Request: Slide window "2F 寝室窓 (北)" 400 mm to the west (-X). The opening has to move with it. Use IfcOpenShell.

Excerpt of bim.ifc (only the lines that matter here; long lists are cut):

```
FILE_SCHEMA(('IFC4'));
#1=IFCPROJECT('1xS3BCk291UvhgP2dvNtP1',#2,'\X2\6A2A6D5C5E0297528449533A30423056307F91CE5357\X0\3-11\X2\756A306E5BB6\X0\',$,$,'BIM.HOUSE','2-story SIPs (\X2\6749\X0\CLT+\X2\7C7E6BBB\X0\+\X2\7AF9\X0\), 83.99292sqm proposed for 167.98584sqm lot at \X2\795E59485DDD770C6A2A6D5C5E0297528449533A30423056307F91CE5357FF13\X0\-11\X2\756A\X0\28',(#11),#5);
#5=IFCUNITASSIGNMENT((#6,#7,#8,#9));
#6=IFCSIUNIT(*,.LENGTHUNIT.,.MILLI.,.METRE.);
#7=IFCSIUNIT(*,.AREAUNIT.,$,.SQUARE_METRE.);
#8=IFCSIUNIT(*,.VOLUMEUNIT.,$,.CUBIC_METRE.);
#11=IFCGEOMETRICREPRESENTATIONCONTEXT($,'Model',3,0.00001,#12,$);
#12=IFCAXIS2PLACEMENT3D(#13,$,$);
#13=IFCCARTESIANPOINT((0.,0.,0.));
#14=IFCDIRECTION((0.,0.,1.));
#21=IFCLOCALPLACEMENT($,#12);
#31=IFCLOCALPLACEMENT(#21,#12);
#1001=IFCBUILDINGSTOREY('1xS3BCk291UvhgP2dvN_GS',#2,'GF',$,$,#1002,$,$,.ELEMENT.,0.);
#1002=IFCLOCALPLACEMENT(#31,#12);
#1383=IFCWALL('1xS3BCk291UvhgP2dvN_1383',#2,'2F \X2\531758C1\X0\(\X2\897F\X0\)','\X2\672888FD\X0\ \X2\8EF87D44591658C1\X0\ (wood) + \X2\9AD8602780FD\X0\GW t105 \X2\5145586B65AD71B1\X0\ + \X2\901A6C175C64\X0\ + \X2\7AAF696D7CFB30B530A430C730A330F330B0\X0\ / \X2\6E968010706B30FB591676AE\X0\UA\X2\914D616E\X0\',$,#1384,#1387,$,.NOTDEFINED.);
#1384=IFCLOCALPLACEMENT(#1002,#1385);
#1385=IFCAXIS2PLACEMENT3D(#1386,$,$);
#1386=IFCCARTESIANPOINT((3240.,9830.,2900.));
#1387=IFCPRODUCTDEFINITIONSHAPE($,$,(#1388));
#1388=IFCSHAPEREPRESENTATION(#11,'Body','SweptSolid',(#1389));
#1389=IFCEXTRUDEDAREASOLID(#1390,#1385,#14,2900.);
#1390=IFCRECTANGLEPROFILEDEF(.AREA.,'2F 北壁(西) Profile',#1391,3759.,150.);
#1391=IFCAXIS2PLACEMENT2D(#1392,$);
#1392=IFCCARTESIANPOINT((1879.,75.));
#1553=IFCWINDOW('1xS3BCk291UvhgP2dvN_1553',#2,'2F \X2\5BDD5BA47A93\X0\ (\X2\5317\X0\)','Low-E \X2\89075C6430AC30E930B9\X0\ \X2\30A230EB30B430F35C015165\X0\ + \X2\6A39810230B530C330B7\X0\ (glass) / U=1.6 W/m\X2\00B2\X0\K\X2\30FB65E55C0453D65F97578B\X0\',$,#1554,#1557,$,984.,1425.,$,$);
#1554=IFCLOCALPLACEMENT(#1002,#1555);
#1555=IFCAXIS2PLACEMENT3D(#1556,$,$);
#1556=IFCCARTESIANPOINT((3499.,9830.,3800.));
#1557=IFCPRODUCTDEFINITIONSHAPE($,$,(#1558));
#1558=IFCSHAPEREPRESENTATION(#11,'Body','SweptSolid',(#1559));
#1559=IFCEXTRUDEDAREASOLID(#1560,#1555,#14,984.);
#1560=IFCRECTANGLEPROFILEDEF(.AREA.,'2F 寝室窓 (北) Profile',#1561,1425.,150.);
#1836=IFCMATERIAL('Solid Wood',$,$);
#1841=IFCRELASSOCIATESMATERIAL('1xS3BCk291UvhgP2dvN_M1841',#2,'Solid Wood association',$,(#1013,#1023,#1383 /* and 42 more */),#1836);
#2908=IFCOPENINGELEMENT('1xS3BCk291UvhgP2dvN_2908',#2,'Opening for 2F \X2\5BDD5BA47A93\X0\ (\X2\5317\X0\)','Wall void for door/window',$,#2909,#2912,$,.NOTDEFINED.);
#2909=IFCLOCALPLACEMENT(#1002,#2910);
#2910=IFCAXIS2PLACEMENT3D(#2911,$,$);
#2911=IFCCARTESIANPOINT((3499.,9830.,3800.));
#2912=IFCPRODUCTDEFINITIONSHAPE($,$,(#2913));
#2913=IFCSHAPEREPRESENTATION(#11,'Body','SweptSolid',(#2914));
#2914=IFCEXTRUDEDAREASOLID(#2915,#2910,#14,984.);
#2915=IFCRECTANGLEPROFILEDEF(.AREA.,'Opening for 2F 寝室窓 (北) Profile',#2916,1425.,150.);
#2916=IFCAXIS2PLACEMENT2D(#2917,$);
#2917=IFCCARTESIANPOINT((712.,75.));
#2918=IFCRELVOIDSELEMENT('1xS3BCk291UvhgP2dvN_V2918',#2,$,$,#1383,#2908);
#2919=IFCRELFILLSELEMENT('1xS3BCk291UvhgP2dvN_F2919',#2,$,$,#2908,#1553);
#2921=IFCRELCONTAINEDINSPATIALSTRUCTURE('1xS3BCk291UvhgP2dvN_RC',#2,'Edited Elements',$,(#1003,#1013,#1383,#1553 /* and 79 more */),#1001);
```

```python
import ifcopenshell
import ifcopenshell.api.geometry
import ifcopenshell.util.placement

model = ifcopenshell.open("bim.ifc")

window = model.by_id(1553)
opening = window.FillsVoids[0].RelatingOpeningElement
wall = opening.VoidsElements[0].RelatingBuildingElement

wall_matrix = ifcopenshell.util.placement.get_local_placement(wall.ObjectPlacement)
shift = wall_matrix[:3, 0] * -400.0
before = ifcopenshell.util.placement.get_local_placement(window.ObjectPlacement)[:3, 3].copy()

# The window is not placed relative to its opening, so move both.
for product in (opening, window):
    matrix = ifcopenshell.util.placement.get_local_placement(product.ObjectPlacement)
    matrix[:3, 3] += shift
    ifcopenshell.api.geometry.edit_object_placement(model, product=product, matrix=matrix, is_si=False)

after = ifcopenshell.util.placement.get_local_placement(window.ObjectPlacement)[:3, 3]
print("window moved by", (after - before).round(3) + 0.0)

model.write("bim-out.ifc")
```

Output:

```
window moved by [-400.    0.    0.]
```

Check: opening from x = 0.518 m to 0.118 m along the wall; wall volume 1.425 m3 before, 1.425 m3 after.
